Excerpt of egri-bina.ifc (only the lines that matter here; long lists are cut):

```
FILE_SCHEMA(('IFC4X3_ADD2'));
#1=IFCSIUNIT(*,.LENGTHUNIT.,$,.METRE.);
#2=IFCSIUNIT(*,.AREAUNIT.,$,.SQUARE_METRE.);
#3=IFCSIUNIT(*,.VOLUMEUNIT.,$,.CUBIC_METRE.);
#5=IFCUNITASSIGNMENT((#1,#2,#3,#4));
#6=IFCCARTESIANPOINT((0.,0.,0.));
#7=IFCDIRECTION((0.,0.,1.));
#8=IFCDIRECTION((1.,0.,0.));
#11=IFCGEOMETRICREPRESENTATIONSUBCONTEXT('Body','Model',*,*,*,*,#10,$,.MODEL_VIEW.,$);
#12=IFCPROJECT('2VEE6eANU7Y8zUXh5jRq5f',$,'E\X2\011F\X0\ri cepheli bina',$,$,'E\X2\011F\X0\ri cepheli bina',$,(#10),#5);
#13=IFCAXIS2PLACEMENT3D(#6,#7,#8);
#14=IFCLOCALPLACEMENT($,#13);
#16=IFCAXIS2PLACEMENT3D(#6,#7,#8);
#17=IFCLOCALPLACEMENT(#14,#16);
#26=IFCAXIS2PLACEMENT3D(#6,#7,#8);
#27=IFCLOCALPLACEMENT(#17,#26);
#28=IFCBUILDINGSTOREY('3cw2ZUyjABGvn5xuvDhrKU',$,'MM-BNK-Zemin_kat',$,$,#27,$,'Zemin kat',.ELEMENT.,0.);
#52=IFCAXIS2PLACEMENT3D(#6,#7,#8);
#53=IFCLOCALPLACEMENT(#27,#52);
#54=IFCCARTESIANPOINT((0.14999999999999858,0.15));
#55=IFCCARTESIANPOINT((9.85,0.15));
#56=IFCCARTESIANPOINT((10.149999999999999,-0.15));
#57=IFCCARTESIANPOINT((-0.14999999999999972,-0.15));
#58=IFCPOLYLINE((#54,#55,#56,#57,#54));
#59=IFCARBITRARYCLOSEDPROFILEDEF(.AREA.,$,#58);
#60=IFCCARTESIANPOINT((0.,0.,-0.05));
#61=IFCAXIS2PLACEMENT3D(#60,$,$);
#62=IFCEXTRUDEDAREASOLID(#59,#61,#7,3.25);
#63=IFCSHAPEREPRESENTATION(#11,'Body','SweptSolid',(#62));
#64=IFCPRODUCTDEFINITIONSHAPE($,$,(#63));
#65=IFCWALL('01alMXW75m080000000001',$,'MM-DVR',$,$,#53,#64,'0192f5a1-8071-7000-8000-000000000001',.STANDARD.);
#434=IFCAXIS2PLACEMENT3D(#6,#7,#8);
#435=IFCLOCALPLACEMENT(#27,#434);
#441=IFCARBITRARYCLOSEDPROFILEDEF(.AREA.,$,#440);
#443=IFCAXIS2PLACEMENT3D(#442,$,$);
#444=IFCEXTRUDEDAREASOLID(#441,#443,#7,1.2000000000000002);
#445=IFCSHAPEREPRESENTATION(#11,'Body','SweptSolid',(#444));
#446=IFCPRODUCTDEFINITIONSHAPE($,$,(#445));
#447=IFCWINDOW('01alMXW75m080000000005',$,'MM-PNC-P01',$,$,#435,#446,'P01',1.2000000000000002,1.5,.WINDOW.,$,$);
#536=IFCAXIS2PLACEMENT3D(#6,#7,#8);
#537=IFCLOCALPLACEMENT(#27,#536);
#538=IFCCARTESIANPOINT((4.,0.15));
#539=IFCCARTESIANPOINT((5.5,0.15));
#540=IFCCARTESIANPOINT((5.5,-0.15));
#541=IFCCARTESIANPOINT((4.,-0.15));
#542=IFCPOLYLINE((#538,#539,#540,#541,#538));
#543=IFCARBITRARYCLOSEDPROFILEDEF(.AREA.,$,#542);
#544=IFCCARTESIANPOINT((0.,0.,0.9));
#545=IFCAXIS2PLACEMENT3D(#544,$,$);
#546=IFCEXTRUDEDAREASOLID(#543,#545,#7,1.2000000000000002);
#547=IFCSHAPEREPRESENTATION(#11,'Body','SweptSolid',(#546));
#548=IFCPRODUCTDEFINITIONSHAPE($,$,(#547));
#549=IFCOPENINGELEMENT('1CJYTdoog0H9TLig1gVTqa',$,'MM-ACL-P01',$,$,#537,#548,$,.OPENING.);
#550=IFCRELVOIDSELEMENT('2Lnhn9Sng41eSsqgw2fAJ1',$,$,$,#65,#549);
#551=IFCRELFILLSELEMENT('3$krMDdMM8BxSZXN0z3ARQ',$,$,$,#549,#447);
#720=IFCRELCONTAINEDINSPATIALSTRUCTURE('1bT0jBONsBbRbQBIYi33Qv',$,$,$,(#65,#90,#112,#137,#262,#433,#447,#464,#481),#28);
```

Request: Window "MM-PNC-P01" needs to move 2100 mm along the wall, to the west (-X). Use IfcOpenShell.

```python
import ifcopenshell
import ifcopenshell.api.geometry
import ifcopenshell.util.placement

model = ifcopenshell.open("egri-bina.ifc")

window = model.by_id(447)
opening = window.FillsVoids[0].RelatingOpeningElement
wall = opening.VoidsElements[0].RelatingBuildingElement

wall_matrix = ifcopenshell.util.placement.get_local_placement(wall.ObjectPlacement)
shift = wall_matrix[:3, 0] * -2.1
before = ifcopenshell.util.placement.get_local_placement(window.ObjectPlacement)[:3, 3].copy()

# The window is not placed relative to its opening, so move both.
for product in (opening, window):
    matrix = ifcopenshell.util.placement.get_local_placement(product.ObjectPlacement)
    matrix[:3, 3] += shift
    ifcopenshell.api.geometry.edit_object_placement(model, product=product, matrix=matrix, is_si=False)

after = ifcopenshell.util.placement.get_local_placement(window.ObjectPlacement)[:3, 3]
print("window moved by", (after - before).round(3) + 0.0)

model.write("egri-bina_updated.ifc")
```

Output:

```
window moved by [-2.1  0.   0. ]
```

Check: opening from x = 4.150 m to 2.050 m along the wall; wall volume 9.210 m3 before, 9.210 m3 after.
